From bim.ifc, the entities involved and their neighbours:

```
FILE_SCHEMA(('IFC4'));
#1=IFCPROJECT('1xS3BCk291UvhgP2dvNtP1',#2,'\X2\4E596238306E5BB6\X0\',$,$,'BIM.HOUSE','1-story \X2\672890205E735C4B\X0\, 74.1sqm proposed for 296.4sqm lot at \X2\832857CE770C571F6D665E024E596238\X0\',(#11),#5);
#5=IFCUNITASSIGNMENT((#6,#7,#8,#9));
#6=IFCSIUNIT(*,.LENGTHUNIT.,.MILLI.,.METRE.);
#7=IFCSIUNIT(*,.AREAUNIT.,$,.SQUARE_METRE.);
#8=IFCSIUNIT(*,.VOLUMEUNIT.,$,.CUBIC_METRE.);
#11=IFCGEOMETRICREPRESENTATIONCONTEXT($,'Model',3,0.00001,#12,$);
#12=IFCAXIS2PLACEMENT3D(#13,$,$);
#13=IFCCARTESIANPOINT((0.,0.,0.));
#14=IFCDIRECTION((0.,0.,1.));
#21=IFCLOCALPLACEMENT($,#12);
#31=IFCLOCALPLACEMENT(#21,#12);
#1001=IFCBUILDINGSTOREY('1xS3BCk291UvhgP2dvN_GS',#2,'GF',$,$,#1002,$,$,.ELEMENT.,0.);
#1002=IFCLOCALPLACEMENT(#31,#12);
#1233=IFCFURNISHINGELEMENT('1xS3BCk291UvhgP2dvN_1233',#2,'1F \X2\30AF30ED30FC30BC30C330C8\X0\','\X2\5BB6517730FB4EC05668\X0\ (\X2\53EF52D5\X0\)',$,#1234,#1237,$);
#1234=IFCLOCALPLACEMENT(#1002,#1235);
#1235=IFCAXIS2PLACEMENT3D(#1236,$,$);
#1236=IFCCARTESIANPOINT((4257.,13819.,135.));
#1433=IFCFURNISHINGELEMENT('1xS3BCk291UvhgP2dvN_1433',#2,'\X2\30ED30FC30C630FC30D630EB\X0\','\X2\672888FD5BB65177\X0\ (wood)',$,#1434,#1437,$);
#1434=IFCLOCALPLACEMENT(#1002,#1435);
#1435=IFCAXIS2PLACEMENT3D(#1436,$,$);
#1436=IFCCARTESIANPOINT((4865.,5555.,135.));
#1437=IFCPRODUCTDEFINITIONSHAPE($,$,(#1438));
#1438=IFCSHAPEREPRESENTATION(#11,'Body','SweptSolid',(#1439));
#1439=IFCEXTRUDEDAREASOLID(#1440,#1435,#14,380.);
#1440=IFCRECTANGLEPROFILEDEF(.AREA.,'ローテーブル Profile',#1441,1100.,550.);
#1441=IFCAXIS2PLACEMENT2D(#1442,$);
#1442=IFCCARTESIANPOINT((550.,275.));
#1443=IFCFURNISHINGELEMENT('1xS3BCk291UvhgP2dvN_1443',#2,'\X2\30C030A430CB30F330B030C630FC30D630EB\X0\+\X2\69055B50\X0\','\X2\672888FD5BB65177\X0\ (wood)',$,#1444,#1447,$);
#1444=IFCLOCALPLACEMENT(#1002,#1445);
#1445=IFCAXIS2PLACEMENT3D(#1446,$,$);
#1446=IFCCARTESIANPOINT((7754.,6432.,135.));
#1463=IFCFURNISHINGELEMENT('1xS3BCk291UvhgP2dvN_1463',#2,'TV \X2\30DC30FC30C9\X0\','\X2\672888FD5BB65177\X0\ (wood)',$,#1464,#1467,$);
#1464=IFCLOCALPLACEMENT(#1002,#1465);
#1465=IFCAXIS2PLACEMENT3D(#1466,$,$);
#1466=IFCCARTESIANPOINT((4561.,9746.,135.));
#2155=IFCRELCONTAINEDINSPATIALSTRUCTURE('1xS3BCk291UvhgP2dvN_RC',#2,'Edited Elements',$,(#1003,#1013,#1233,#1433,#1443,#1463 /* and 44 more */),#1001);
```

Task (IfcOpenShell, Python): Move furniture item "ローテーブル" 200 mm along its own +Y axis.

```python
import ifcopenshell
import ifcopenshell.api.geometry
import ifcopenshell.util.placement

model = ifcopenshell.open("bim.ifc")

item = model.by_guid("1xS3BCk291UvhgP2dvN_1433")
matrix = ifcopenshell.util.placement.get_local_placement(item.ObjectPlacement)
matrix[:3, 3] += matrix[:3, 1] * 200.0
ifcopenshell.api.geometry.edit_object_placement(model, product=item, matrix=matrix, is_si=False)

print(ifcopenshell.util.placement.get_local_placement(item.ObjectPlacement).round(3) + 0.0)

model.write("bim-out.ifc")
```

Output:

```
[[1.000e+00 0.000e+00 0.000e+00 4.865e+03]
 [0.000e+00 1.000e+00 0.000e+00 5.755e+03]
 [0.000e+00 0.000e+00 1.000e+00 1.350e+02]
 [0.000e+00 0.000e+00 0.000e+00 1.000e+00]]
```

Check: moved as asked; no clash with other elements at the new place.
